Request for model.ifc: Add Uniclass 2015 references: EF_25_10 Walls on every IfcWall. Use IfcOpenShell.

First a look at what the model holds.

```python
import ifcopenshell

model = ifcopenshell.open("model.ifc")
print(model.schema)
print("classifications:", [c.Name for c in model.by_type("IfcClassification")])
for ifc_class in ("IfcDoor", "IfcRoof", "IfcStair", "IfcWall", "IfcWindow"):
    print(ifc_class, len(model.by_type(ifc_class)))
```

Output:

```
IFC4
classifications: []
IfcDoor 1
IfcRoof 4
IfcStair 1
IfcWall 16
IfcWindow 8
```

```python
import ifcopenshell
import ifcopenshell.api.classification

model = ifcopenshell.open("model.ifc")

system = ifcopenshell.api.classification.add_classification(model, classification="Uniclass 2015")

codes = {
    "IfcWall": ("EF_25_10", "Walls"),
}
for ifc_class, (code, name) in codes.items():
    products = model.by_type(ifc_class)
    ifcopenshell.api.classification.add_reference(
        model, products=products, classification=system, identification=code, name=name
    )
    print(code, len(products))

model.write("model-out.ifc")
```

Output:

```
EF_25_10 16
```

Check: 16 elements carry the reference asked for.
